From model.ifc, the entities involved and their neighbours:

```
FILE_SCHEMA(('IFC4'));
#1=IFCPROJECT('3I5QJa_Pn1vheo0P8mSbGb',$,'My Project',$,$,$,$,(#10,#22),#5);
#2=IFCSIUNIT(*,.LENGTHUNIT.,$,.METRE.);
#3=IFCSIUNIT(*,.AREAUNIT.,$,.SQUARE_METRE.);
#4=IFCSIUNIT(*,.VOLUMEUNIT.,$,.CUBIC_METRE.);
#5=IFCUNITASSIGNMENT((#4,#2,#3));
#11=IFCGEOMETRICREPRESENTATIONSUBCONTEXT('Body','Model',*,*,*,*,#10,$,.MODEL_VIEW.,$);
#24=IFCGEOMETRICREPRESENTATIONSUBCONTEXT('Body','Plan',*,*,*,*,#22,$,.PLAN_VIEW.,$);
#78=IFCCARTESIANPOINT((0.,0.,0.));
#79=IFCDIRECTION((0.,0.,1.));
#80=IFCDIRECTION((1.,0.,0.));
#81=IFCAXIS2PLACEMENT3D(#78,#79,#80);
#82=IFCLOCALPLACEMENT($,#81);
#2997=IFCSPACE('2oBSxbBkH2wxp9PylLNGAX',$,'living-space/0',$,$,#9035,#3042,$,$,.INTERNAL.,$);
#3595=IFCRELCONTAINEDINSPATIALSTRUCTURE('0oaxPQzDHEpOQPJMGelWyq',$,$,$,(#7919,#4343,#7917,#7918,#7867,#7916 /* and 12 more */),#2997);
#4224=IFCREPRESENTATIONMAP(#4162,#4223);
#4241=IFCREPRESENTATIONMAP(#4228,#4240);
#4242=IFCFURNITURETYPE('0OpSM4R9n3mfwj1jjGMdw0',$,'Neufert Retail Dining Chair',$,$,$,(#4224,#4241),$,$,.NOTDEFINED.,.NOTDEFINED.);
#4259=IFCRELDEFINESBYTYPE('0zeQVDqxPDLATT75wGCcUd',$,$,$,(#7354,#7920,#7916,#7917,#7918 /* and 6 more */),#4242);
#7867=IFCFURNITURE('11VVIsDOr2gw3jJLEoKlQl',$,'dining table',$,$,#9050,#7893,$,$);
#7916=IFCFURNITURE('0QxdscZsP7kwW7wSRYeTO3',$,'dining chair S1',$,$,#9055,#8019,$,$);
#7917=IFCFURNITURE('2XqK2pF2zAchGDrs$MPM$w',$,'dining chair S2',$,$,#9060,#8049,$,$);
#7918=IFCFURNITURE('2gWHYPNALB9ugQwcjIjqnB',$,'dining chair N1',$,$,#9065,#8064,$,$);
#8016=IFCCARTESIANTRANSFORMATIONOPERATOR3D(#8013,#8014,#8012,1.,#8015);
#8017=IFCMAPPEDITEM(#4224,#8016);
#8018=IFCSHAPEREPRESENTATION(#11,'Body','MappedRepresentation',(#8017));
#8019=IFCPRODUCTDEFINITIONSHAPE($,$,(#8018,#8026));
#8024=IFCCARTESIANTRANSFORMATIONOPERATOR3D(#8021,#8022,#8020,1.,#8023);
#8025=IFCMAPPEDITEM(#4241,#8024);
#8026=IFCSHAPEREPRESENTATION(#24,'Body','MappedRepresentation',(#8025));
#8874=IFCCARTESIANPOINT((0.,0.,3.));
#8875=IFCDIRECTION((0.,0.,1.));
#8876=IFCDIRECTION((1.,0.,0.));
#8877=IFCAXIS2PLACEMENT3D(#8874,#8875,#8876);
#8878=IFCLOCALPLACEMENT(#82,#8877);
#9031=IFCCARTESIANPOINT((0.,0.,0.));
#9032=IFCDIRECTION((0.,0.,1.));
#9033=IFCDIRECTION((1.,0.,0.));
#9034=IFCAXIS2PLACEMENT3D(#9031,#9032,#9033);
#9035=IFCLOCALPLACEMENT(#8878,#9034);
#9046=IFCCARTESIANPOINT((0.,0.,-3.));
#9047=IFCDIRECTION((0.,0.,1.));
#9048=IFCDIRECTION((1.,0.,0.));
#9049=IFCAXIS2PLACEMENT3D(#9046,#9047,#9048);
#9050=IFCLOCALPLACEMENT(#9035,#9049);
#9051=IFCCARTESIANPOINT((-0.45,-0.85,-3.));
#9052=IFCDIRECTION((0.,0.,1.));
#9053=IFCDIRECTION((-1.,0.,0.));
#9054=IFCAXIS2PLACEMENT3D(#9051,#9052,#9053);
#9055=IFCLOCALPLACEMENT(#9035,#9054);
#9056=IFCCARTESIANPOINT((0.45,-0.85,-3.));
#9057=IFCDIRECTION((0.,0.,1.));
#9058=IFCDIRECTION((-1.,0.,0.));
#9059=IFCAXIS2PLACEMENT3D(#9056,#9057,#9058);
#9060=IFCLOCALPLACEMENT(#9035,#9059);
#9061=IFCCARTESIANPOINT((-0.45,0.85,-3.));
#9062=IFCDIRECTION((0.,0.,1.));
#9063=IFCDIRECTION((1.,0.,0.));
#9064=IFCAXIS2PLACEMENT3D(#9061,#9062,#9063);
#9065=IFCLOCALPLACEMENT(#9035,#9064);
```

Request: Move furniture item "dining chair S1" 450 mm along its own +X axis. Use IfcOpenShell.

```python
import ifcopenshell
import ifcopenshell.api.geometry
import ifcopenshell.util.placement

model = ifcopenshell.open("model.ifc")

item = model.by_guid("0QxdscZsP7kwW7wSRYeTO3")
matrix = ifcopenshell.util.placement.get_local_placement(item.ObjectPlacement)
matrix[:3, 3] += matrix[:3, 0] * 0.45
ifcopenshell.api.geometry.edit_object_placement(model, product=item, matrix=matrix, is_si=False)

print(ifcopenshell.util.placement.get_local_placement(item.ObjectPlacement).round(3) + 0.0)

model.write("model_updated.ifc")
```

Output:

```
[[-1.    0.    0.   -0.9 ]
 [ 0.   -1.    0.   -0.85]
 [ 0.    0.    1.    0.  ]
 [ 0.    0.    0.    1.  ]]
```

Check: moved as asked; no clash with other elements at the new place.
